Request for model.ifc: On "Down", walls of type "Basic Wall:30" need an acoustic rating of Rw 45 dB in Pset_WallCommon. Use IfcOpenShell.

First a look at what the model holds.

```python
import ifcopenshell
import ifcopenshell.util.element

model = ifcopenshell.open("model.ifc")
print(model.schema)
storey = next(s for s in model.by_type("IfcBuildingStorey") if s.Name == "Down")
walls = [e for e in ifcopenshell.util.element.get_decomposition(storey) if e.is_a("IfcWall")]
seen = {}
for e in walls:
    element_type = ifcopenshell.util.element.get_type(e)
    key = (element_type.Name if element_type != e and element_type else None, ifcopenshell.util.element.get_pset(e, "Pset_WallCommon", "AcousticRating"))
    seen[key] = seen.get(key, 0) + 1
for (name, value), count in sorted(seen.items(), key=str):
    print(count, "x", name, "|", value)
```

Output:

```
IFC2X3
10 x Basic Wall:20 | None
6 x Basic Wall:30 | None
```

```python
import ifcopenshell
import ifcopenshell.api.pset
import ifcopenshell.util.element

model = ifcopenshell.open("model.ifc")

storey = next(s for s in model.by_type("IfcBuildingStorey") if s.Name == "Down")
walls = [e for e in ifcopenshell.util.element.get_decomposition(storey) if e.is_a("IfcWall")]

count = 0
for e in walls:
    element_type = ifcopenshell.util.element.get_type(e)
    if element_type in (None, e) or element_type.Name != "Basic Wall:30":
        continue
    # add_pset returns the element's existing set when there is one.
    pset = ifcopenshell.api.pset.add_pset(model, product=e, name="Pset_WallCommon")
    ifcopenshell.api.pset.edit_pset(model, pset=pset, properties={"AcousticRating": "Rw 45 dB"})
    count += 1

print(count, "walls updated")

model.write("model_v2.ifc")
```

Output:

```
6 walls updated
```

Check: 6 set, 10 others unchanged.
